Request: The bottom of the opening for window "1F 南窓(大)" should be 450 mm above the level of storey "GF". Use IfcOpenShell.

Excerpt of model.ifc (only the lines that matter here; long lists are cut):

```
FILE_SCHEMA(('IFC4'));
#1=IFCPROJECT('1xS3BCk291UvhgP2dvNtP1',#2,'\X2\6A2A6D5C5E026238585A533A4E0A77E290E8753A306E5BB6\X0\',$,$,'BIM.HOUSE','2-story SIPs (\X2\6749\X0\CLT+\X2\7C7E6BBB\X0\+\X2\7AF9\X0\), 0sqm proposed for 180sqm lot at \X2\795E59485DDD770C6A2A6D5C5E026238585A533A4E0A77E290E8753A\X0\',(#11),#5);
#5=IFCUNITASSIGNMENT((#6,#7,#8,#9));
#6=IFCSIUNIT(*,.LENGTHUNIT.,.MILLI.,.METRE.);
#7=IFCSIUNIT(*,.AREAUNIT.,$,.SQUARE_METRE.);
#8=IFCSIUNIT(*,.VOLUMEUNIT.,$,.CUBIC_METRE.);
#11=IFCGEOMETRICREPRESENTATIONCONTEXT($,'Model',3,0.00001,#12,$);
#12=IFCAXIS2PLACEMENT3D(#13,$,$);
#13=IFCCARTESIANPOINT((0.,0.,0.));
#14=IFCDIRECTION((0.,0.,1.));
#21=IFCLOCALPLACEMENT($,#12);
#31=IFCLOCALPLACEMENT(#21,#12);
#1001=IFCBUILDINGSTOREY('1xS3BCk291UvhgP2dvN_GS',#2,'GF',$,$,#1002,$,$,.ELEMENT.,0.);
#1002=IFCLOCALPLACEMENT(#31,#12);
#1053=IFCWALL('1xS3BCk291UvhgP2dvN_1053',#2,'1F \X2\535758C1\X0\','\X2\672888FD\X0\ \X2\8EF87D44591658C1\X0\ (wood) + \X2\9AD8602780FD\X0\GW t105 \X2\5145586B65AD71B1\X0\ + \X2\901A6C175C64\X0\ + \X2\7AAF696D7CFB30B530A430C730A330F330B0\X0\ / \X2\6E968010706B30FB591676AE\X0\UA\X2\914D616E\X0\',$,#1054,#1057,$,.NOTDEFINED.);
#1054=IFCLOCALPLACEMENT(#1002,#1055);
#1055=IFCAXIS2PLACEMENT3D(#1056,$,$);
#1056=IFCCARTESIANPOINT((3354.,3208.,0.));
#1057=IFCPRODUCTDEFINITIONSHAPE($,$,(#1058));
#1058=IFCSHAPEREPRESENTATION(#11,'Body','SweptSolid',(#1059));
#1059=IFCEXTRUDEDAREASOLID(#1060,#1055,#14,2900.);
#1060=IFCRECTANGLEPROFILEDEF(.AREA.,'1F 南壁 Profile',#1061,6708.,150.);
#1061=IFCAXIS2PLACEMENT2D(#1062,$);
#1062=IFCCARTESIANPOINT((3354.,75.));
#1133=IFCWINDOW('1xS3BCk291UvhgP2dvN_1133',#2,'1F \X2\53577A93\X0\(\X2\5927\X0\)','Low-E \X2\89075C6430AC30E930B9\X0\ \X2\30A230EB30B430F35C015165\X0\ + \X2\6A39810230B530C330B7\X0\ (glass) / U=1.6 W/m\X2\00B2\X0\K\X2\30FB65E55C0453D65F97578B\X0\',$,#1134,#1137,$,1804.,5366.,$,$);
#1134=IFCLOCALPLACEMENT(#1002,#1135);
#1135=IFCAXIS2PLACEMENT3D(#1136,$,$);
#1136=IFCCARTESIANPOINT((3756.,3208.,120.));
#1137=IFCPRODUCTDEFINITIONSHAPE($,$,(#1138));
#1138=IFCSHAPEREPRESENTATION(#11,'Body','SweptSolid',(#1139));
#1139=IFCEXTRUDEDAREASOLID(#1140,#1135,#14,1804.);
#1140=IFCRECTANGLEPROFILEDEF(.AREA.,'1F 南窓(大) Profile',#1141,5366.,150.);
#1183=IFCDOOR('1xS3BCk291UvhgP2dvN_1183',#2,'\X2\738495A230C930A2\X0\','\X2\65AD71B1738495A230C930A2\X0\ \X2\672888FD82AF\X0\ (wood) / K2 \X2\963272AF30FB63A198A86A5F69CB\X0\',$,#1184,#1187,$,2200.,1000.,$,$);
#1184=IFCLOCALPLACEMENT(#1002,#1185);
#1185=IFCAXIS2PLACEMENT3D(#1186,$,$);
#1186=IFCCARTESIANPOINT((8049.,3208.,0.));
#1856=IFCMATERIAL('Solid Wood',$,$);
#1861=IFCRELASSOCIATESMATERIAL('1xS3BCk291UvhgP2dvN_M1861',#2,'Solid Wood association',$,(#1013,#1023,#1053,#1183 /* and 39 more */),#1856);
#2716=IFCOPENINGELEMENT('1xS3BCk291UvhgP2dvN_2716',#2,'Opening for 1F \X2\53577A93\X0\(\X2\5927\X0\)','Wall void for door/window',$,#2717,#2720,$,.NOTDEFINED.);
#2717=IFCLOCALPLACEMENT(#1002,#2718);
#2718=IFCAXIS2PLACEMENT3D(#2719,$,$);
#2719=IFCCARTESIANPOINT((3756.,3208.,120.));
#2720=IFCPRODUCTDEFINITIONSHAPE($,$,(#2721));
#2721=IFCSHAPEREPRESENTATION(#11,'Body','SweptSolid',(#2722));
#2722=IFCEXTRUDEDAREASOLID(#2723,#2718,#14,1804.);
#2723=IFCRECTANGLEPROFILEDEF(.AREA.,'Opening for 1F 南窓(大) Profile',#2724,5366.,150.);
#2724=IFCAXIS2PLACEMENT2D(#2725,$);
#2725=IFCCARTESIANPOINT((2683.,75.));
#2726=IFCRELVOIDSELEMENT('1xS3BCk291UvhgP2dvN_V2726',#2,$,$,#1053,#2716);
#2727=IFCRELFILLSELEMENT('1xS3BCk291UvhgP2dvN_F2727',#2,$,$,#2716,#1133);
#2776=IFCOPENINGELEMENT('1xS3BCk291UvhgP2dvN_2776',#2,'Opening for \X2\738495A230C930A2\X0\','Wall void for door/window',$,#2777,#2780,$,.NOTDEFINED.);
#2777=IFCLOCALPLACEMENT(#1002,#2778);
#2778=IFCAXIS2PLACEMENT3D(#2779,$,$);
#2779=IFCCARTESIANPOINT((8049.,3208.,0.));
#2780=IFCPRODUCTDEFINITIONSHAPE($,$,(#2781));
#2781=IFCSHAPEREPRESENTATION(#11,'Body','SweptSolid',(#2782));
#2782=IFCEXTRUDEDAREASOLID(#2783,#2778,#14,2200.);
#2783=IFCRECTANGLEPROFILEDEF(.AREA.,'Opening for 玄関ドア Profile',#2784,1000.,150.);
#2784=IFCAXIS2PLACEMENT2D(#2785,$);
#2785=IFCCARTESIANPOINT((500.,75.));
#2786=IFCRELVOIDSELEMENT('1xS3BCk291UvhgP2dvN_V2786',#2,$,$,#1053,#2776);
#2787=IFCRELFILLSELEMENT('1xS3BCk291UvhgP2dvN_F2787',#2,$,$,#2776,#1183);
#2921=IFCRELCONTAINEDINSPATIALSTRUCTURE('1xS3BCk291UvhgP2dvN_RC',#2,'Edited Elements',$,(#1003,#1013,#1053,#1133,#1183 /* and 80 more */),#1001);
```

```python
import numpy as np
import ifcopenshell
import ifcopenshell.api.geometry
import ifcopenshell.geom
import ifcopenshell.util.element
import ifcopenshell.util.placement
import ifcopenshell.util.shape
import ifcopenshell.util.unit

model = ifcopenshell.open("model.ifc")
unit_scale = ifcopenshell.util.unit.calculate_unit_scale(model)

window = model.by_id(1133)
opening = window.FillsVoids[0].RelatingOpeningElement
storey = ifcopenshell.util.element.get_container(window, ifc_class="IfcBuildingStorey")
level = ifcopenshell.util.placement.get_local_placement(storey.ObjectPlacement)[2, 3]

# The opening's origin need not be at the sill, so measure its lowest point.
shape = ifcopenshell.geom.create_shape(ifcopenshell.geom.settings(), opening)
bottom = ifcopenshell.util.shape.get_shape_bottom_elevation(shape, shape.geometry) / unit_scale
dz = level + 0.45 / unit_scale - bottom

shift = np.array([0.0, 0.0, dz])
# The window is not placed relative to its opening, so move both.
for product in (opening, window):
    matrix = ifcopenshell.util.placement.get_local_placement(product.ObjectPlacement)
    matrix[:3, 3] += shift
    ifcopenshell.api.geometry.edit_object_placement(model, product=product, matrix=matrix, is_si=False)

print(f"moved by {dz * unit_scale:+.3f} m")

model.write("model_updated.ifc")
```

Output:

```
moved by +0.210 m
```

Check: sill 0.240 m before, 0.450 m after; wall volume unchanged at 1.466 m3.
